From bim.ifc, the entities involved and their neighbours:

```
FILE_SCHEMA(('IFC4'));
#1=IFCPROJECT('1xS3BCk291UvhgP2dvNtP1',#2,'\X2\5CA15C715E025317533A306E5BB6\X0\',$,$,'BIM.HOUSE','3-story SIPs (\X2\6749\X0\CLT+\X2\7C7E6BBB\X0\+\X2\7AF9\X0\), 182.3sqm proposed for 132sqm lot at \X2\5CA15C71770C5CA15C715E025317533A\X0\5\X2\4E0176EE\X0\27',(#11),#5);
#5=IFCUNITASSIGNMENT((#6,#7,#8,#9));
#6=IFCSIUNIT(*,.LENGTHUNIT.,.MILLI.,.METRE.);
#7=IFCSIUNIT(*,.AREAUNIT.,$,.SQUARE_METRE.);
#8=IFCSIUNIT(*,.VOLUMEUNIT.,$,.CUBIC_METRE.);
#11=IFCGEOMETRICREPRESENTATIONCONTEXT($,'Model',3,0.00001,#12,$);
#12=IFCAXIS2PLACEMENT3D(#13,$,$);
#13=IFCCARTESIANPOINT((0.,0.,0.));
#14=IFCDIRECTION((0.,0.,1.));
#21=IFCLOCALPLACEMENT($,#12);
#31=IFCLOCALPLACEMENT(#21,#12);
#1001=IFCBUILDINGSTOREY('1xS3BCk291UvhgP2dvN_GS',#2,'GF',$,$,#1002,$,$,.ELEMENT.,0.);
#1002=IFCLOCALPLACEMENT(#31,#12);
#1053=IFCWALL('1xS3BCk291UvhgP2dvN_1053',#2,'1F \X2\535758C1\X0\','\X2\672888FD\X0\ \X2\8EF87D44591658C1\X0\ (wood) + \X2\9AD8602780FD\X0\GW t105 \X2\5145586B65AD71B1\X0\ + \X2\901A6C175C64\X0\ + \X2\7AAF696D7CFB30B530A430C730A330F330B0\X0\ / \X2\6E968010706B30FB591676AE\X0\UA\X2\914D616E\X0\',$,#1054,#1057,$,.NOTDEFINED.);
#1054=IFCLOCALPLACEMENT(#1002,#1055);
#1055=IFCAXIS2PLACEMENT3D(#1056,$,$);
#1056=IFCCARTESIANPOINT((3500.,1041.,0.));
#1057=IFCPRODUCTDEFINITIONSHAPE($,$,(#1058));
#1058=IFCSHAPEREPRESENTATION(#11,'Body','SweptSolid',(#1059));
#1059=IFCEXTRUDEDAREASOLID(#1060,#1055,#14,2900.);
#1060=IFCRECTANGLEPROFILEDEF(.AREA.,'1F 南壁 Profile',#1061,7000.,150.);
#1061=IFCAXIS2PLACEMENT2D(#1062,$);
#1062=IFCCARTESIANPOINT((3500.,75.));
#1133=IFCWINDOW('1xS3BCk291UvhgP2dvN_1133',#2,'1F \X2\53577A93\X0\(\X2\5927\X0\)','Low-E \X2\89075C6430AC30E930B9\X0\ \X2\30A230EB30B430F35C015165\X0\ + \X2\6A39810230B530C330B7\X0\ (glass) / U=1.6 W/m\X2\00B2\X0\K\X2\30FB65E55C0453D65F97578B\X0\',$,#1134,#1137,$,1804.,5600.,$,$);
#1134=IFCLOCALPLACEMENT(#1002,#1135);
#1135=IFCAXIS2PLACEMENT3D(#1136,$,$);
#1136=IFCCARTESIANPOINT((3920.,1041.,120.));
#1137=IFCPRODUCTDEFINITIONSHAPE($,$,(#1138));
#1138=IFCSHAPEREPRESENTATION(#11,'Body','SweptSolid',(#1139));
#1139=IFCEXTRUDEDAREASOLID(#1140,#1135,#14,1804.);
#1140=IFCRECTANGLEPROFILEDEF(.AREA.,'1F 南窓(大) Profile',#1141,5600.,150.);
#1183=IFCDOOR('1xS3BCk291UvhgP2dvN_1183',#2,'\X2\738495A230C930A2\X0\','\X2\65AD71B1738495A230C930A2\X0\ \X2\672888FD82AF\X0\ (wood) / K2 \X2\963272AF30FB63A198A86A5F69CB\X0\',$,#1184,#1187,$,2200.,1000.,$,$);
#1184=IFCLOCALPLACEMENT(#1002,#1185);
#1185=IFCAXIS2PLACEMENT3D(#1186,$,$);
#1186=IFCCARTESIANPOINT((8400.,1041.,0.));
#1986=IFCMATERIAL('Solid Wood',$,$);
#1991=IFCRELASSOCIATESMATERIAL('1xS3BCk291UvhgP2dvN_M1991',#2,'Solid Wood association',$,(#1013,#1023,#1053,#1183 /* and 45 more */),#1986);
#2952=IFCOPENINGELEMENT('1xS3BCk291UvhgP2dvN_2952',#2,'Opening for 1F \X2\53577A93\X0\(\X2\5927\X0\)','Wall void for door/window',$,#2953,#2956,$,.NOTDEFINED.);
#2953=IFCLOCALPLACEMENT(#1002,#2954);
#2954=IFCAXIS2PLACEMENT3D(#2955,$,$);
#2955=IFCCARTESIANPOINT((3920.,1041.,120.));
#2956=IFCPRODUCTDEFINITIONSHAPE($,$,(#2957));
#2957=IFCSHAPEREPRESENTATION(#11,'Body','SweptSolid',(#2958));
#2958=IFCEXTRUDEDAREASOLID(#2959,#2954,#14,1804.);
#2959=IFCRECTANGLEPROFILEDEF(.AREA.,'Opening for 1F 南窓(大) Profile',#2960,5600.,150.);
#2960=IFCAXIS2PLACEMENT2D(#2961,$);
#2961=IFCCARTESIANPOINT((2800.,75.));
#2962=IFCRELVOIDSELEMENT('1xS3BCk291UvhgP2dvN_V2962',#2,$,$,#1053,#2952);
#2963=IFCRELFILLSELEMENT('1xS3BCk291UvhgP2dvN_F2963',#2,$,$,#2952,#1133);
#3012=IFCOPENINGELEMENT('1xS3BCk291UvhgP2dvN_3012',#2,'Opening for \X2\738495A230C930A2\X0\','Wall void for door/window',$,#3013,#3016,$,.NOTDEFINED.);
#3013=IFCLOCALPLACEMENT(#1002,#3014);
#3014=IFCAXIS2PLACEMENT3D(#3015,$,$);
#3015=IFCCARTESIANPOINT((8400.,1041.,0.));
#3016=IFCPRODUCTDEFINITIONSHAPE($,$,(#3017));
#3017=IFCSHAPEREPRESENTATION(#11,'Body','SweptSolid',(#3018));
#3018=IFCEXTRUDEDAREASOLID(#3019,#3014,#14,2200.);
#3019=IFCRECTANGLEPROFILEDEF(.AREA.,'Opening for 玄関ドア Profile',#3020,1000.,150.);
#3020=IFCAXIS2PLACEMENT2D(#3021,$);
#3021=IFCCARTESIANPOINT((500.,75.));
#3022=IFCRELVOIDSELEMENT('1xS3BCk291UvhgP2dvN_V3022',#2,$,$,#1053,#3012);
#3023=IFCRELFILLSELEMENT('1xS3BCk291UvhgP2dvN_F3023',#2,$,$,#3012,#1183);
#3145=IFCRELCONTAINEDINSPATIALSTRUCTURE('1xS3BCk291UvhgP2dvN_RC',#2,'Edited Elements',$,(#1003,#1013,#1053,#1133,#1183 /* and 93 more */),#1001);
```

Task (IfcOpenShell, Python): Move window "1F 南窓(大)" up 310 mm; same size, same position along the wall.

```python
import numpy as np
import ifcopenshell
import ifcopenshell.api.geometry
import ifcopenshell.util.placement
import ifcopenshell.util.unit

model = ifcopenshell.open("bim.ifc")
unit_scale = ifcopenshell.util.unit.calculate_unit_scale(model)

window = model.by_guid("1xS3BCk291UvhgP2dvN_1133")
opening = window.FillsVoids[0].RelatingOpeningElement
dz = 0.31 / unit_scale

shift = np.array([0.0, 0.0, dz])
# The window is not placed relative to its opening, so move both.
for product in (opening, window):
    matrix = ifcopenshell.util.placement.get_local_placement(product.ObjectPlacement)
    matrix[:3, 3] += shift
    ifcopenshell.api.geometry.edit_object_placement(model, product=product, matrix=matrix, is_si=False)

print(f"moved by {dz * unit_scale:+.3f} m")

model.write("bim_v2.ifc")
```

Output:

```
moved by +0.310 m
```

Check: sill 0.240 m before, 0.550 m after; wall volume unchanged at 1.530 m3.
